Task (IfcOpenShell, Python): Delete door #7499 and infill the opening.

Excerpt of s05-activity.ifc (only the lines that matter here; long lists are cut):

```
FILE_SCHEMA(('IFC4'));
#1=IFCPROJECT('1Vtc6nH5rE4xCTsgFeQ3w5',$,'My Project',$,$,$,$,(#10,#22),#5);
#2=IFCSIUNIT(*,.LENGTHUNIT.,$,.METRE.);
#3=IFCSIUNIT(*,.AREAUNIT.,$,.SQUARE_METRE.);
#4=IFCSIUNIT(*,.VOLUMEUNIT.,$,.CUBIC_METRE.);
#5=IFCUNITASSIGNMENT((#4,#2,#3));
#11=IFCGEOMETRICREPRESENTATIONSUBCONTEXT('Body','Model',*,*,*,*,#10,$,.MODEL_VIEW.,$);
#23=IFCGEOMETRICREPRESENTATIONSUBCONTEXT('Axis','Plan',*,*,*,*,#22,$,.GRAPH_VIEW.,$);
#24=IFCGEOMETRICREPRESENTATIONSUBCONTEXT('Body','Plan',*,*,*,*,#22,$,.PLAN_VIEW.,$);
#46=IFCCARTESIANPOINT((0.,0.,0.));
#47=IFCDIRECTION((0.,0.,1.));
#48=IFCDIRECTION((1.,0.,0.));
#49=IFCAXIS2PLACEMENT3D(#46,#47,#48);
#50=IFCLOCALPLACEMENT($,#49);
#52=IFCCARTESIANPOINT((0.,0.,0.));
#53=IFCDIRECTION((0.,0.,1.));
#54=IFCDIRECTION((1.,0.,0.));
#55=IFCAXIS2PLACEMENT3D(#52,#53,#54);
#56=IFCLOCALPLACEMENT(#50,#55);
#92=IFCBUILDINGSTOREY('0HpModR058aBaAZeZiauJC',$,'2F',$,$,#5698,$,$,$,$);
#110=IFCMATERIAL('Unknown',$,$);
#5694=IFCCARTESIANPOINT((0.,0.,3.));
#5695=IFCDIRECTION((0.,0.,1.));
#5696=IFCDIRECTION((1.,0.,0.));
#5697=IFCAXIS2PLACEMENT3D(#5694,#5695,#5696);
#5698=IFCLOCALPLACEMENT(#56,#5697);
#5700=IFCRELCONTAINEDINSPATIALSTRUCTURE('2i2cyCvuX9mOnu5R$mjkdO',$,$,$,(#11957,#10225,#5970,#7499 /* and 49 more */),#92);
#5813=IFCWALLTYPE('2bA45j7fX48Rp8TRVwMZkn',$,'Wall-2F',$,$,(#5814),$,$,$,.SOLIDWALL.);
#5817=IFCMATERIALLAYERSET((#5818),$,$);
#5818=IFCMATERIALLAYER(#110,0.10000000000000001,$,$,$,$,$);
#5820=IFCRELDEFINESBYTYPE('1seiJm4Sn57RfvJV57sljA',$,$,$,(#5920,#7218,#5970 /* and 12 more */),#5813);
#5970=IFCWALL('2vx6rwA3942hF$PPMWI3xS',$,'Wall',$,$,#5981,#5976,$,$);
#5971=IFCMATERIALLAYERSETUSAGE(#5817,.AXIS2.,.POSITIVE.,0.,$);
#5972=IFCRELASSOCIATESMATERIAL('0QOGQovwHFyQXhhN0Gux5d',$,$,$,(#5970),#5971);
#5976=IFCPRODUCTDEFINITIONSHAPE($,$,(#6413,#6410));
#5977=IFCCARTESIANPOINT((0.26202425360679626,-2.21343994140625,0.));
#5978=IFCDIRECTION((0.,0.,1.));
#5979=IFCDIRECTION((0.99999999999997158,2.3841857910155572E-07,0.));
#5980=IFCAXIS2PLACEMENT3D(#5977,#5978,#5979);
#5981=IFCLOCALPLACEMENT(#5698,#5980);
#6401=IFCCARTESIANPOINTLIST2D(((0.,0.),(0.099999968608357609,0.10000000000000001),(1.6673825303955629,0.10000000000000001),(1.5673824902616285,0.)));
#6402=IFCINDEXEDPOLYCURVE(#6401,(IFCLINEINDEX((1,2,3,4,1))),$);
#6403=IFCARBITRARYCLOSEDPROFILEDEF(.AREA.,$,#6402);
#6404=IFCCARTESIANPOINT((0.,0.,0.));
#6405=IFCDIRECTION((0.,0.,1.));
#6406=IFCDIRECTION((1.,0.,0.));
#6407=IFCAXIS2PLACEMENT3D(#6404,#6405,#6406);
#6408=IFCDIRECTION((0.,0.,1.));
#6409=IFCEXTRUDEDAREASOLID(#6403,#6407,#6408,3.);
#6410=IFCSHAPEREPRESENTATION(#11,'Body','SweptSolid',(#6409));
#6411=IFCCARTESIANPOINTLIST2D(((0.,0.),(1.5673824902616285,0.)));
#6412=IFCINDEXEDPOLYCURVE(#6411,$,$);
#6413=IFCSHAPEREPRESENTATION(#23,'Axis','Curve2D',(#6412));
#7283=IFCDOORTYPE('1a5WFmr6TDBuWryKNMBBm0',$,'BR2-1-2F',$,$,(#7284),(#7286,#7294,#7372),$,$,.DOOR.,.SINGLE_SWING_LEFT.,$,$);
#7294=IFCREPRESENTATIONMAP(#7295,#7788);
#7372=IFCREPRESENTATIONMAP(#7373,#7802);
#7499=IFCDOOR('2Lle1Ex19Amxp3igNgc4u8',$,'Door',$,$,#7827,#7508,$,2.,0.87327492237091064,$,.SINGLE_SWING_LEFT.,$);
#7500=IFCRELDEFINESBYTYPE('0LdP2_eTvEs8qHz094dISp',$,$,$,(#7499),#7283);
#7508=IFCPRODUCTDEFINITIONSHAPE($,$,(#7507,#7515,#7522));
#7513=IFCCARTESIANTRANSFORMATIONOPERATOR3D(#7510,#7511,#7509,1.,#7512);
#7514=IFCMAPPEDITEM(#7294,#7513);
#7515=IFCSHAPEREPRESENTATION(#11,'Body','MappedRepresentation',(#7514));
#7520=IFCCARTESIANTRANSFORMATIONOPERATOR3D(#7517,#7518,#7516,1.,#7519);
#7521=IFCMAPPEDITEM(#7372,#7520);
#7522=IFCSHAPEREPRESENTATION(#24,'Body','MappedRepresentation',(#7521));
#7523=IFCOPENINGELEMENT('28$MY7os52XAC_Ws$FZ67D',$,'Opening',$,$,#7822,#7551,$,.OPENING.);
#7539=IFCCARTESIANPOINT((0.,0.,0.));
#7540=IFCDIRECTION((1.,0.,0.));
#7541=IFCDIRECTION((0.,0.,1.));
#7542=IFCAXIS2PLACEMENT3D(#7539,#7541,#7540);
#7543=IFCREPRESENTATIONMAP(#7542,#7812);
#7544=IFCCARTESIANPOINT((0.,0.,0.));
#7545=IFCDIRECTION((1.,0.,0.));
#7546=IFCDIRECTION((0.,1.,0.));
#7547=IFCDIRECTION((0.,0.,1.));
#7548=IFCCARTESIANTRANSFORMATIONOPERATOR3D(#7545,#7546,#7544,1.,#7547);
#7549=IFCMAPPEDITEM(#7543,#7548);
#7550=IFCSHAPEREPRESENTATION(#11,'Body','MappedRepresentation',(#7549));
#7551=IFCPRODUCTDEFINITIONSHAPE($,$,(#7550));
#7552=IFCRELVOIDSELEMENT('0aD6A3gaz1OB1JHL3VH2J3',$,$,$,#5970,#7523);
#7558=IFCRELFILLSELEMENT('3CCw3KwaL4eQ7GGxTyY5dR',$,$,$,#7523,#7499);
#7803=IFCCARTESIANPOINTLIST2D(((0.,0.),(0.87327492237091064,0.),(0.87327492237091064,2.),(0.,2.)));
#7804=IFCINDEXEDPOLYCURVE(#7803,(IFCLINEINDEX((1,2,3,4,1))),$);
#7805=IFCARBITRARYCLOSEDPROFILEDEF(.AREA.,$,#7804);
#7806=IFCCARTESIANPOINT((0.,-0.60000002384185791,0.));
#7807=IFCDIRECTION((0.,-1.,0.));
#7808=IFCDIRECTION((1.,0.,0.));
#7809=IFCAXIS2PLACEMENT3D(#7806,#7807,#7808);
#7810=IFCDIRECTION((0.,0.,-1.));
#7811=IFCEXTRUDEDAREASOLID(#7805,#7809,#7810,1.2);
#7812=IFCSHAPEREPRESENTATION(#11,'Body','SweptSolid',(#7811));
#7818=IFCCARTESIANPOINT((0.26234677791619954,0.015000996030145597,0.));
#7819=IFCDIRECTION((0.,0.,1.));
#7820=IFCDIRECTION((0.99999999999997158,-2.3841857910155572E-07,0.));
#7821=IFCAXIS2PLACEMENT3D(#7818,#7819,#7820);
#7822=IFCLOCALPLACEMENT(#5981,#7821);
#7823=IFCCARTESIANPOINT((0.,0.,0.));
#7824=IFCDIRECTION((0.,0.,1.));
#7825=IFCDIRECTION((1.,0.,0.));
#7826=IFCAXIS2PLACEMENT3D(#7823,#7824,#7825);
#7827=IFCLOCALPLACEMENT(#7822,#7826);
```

```python
import ifcopenshell
import ifcopenshell.api.feature
import ifcopenshell.api.root
import ifcopenshell.geom
import ifcopenshell.util.shape

model = ifcopenshell.open("s05-activity.ifc")
settings = ifcopenshell.geom.settings()


def volume(element):
    """Net volume in cubic metres, openings subtracted."""
    shape = ifcopenshell.geom.create_shape(settings, element)
    return ifcopenshell.util.shape.get_volume(shape.geometry)


door = model.by_guid("2Lle1Ex19Amxp3igNgc4u8")
opening = door.FillsVoids[0].RelatingOpeningElement
wall = opening.VoidsElements[0].RelatingBuildingElement
before = volume(wall)

ifcopenshell.api.root.remove_product(model, product=door)
ifcopenshell.api.feature.remove_feature(model, feature=opening)

after = volume(wall)

print(f"wall volume {before:.3f} -> {after:.3f} m3")

model.write("s05-activity_rev.ifc")
```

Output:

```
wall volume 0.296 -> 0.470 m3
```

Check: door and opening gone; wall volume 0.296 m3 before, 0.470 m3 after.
